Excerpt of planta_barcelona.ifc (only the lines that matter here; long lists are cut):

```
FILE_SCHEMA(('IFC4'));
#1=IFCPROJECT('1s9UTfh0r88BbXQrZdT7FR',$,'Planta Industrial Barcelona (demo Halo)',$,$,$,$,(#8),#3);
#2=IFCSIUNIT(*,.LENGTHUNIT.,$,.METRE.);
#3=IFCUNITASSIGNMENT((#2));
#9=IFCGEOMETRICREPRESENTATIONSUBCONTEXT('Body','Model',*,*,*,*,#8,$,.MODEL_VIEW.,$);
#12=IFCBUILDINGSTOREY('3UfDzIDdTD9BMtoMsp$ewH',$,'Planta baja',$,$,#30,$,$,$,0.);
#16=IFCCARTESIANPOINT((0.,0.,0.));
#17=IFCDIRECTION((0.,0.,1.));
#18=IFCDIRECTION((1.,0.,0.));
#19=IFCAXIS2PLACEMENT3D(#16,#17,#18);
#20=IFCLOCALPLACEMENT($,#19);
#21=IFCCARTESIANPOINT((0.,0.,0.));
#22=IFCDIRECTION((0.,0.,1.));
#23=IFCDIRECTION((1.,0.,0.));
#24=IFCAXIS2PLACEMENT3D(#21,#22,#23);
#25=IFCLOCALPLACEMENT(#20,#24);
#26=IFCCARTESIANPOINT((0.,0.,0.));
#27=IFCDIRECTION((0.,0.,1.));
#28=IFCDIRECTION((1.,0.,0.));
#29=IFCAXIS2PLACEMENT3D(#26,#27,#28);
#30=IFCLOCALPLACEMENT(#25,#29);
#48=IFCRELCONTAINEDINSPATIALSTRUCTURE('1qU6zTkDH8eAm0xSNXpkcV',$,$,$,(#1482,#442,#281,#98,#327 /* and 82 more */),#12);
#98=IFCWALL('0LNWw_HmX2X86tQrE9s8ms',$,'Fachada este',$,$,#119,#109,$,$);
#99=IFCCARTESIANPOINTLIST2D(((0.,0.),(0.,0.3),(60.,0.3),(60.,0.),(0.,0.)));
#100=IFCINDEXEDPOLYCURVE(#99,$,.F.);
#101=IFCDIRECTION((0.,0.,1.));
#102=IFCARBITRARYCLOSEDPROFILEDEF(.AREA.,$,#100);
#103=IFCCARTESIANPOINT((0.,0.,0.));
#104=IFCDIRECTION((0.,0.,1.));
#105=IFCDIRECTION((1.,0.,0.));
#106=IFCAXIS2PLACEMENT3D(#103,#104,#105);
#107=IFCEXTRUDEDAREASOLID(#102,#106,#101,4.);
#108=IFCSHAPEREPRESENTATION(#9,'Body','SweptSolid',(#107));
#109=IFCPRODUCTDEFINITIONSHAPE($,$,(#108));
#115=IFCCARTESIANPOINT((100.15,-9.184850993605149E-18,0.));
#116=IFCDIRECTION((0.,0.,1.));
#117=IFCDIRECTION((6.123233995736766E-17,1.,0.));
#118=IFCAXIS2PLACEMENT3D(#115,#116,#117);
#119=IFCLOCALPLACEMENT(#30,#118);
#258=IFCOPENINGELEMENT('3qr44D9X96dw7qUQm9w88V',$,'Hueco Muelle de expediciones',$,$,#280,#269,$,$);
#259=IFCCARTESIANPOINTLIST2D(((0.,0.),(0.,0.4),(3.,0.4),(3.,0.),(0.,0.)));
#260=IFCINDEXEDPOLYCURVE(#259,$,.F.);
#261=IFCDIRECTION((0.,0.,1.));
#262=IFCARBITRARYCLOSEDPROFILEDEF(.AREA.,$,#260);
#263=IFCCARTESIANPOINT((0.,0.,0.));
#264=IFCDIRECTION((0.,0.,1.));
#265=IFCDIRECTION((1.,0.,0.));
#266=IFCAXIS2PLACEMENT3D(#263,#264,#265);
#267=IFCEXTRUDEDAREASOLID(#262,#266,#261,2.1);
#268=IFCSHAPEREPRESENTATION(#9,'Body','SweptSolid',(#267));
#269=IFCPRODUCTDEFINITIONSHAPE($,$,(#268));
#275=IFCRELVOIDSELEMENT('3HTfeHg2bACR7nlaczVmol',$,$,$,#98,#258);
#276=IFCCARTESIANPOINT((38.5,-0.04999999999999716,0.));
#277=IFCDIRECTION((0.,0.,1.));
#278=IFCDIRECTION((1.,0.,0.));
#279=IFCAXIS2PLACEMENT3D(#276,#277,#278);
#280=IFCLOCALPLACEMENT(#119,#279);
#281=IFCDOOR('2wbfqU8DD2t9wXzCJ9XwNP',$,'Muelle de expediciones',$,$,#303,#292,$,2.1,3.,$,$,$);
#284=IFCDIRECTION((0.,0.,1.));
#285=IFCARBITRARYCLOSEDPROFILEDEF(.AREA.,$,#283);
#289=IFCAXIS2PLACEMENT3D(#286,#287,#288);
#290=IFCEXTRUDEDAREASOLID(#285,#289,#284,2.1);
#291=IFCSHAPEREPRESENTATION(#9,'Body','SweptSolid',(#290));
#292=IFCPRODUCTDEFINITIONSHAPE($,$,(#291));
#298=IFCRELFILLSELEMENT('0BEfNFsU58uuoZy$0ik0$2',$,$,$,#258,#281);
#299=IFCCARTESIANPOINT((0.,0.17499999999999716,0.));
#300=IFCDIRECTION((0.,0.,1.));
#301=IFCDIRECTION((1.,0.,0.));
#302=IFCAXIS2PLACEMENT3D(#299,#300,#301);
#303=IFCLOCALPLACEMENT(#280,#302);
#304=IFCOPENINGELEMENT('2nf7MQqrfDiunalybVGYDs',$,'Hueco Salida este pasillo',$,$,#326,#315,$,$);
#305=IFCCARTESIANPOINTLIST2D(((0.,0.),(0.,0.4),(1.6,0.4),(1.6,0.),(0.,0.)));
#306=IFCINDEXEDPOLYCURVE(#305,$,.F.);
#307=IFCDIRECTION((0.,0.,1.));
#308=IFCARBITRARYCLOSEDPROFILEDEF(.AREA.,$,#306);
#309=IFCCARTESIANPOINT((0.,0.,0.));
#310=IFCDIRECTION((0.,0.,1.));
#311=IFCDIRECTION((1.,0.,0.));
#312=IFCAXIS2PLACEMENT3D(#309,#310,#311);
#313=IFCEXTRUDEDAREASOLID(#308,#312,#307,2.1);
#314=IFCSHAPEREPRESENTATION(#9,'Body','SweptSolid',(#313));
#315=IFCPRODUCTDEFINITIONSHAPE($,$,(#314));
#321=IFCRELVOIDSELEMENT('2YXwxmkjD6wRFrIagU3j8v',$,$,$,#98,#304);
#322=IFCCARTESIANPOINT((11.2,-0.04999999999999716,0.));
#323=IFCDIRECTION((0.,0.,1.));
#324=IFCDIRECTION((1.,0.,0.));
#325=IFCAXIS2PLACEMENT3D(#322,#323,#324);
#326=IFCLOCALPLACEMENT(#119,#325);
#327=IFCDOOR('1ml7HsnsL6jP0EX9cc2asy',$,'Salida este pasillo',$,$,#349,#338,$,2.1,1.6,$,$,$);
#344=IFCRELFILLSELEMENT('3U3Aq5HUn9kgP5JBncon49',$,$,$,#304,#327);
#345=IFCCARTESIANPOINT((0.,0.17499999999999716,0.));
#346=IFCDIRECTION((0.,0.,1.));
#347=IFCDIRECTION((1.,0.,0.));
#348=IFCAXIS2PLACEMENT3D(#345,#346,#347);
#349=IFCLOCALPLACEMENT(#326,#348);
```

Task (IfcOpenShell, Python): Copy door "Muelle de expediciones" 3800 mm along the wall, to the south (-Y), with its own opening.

```python
import ifcopenshell
import ifcopenshell.api.feature
import ifcopenshell.api.geometry
import ifcopenshell.api.root
import ifcopenshell.geom
import ifcopenshell.util.element
import ifcopenshell.util.placement
import ifcopenshell.util.shape
import ifcopenshell.util.unit

model = ifcopenshell.open("planta_barcelona.ifc")
unit_scale = ifcopenshell.util.unit.calculate_unit_scale(model)
settings = ifcopenshell.geom.settings()


def volume(element):
    """Net volume in cubic metres, openings subtracted."""
    shape = ifcopenshell.geom.create_shape(settings, element)
    return ifcopenshell.util.shape.get_volume(shape.geometry)


door = model.by_guid("2wbfqU8DD2t9wXzCJ9XwNP")
opening = door.FillsVoids[0].RelatingOpeningElement
wall = opening.VoidsElements[0].RelatingBuildingElement
before = volume(wall)
shift = ifcopenshell.util.placement.get_local_placement(wall.ObjectPlacement)[:3, 0] * -3.8 / unit_scale

# copy_class copies the void relationship, type, container and properties, but no geometry.
new_opening = ifcopenshell.api.root.copy_class(model, product=opening)
new_opening.Representation = ifcopenshell.util.element.copy_deep(
    model, opening.Representation, exclude=["IfcGeometricRepresentationContext", "IfcRepresentationMap"]
)
new_door = ifcopenshell.api.root.copy_class(model, product=door)
new_door.Representation = ifcopenshell.util.element.copy_deep(
    model, door.Representation, exclude=["IfcGeometricRepresentationContext", "IfcRepresentationMap"]
)
ifcopenshell.api.feature.add_filling(model, opening=new_opening, element=new_door)

for old, new in ((opening, new_opening), (door, new_door)):
    matrix = ifcopenshell.util.placement.get_local_placement(old.ObjectPlacement)
    matrix[:3, 3] += shift
    ifcopenshell.api.geometry.edit_object_placement(model, product=new, matrix=matrix, is_si=False)

after = volume(wall)

print(f"wall volume {before:.3f} -> {after:.3f} m3")

model.write("planta_barcelona_rev.ifc")
```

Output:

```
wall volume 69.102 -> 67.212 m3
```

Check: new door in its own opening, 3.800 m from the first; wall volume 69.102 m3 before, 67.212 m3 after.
